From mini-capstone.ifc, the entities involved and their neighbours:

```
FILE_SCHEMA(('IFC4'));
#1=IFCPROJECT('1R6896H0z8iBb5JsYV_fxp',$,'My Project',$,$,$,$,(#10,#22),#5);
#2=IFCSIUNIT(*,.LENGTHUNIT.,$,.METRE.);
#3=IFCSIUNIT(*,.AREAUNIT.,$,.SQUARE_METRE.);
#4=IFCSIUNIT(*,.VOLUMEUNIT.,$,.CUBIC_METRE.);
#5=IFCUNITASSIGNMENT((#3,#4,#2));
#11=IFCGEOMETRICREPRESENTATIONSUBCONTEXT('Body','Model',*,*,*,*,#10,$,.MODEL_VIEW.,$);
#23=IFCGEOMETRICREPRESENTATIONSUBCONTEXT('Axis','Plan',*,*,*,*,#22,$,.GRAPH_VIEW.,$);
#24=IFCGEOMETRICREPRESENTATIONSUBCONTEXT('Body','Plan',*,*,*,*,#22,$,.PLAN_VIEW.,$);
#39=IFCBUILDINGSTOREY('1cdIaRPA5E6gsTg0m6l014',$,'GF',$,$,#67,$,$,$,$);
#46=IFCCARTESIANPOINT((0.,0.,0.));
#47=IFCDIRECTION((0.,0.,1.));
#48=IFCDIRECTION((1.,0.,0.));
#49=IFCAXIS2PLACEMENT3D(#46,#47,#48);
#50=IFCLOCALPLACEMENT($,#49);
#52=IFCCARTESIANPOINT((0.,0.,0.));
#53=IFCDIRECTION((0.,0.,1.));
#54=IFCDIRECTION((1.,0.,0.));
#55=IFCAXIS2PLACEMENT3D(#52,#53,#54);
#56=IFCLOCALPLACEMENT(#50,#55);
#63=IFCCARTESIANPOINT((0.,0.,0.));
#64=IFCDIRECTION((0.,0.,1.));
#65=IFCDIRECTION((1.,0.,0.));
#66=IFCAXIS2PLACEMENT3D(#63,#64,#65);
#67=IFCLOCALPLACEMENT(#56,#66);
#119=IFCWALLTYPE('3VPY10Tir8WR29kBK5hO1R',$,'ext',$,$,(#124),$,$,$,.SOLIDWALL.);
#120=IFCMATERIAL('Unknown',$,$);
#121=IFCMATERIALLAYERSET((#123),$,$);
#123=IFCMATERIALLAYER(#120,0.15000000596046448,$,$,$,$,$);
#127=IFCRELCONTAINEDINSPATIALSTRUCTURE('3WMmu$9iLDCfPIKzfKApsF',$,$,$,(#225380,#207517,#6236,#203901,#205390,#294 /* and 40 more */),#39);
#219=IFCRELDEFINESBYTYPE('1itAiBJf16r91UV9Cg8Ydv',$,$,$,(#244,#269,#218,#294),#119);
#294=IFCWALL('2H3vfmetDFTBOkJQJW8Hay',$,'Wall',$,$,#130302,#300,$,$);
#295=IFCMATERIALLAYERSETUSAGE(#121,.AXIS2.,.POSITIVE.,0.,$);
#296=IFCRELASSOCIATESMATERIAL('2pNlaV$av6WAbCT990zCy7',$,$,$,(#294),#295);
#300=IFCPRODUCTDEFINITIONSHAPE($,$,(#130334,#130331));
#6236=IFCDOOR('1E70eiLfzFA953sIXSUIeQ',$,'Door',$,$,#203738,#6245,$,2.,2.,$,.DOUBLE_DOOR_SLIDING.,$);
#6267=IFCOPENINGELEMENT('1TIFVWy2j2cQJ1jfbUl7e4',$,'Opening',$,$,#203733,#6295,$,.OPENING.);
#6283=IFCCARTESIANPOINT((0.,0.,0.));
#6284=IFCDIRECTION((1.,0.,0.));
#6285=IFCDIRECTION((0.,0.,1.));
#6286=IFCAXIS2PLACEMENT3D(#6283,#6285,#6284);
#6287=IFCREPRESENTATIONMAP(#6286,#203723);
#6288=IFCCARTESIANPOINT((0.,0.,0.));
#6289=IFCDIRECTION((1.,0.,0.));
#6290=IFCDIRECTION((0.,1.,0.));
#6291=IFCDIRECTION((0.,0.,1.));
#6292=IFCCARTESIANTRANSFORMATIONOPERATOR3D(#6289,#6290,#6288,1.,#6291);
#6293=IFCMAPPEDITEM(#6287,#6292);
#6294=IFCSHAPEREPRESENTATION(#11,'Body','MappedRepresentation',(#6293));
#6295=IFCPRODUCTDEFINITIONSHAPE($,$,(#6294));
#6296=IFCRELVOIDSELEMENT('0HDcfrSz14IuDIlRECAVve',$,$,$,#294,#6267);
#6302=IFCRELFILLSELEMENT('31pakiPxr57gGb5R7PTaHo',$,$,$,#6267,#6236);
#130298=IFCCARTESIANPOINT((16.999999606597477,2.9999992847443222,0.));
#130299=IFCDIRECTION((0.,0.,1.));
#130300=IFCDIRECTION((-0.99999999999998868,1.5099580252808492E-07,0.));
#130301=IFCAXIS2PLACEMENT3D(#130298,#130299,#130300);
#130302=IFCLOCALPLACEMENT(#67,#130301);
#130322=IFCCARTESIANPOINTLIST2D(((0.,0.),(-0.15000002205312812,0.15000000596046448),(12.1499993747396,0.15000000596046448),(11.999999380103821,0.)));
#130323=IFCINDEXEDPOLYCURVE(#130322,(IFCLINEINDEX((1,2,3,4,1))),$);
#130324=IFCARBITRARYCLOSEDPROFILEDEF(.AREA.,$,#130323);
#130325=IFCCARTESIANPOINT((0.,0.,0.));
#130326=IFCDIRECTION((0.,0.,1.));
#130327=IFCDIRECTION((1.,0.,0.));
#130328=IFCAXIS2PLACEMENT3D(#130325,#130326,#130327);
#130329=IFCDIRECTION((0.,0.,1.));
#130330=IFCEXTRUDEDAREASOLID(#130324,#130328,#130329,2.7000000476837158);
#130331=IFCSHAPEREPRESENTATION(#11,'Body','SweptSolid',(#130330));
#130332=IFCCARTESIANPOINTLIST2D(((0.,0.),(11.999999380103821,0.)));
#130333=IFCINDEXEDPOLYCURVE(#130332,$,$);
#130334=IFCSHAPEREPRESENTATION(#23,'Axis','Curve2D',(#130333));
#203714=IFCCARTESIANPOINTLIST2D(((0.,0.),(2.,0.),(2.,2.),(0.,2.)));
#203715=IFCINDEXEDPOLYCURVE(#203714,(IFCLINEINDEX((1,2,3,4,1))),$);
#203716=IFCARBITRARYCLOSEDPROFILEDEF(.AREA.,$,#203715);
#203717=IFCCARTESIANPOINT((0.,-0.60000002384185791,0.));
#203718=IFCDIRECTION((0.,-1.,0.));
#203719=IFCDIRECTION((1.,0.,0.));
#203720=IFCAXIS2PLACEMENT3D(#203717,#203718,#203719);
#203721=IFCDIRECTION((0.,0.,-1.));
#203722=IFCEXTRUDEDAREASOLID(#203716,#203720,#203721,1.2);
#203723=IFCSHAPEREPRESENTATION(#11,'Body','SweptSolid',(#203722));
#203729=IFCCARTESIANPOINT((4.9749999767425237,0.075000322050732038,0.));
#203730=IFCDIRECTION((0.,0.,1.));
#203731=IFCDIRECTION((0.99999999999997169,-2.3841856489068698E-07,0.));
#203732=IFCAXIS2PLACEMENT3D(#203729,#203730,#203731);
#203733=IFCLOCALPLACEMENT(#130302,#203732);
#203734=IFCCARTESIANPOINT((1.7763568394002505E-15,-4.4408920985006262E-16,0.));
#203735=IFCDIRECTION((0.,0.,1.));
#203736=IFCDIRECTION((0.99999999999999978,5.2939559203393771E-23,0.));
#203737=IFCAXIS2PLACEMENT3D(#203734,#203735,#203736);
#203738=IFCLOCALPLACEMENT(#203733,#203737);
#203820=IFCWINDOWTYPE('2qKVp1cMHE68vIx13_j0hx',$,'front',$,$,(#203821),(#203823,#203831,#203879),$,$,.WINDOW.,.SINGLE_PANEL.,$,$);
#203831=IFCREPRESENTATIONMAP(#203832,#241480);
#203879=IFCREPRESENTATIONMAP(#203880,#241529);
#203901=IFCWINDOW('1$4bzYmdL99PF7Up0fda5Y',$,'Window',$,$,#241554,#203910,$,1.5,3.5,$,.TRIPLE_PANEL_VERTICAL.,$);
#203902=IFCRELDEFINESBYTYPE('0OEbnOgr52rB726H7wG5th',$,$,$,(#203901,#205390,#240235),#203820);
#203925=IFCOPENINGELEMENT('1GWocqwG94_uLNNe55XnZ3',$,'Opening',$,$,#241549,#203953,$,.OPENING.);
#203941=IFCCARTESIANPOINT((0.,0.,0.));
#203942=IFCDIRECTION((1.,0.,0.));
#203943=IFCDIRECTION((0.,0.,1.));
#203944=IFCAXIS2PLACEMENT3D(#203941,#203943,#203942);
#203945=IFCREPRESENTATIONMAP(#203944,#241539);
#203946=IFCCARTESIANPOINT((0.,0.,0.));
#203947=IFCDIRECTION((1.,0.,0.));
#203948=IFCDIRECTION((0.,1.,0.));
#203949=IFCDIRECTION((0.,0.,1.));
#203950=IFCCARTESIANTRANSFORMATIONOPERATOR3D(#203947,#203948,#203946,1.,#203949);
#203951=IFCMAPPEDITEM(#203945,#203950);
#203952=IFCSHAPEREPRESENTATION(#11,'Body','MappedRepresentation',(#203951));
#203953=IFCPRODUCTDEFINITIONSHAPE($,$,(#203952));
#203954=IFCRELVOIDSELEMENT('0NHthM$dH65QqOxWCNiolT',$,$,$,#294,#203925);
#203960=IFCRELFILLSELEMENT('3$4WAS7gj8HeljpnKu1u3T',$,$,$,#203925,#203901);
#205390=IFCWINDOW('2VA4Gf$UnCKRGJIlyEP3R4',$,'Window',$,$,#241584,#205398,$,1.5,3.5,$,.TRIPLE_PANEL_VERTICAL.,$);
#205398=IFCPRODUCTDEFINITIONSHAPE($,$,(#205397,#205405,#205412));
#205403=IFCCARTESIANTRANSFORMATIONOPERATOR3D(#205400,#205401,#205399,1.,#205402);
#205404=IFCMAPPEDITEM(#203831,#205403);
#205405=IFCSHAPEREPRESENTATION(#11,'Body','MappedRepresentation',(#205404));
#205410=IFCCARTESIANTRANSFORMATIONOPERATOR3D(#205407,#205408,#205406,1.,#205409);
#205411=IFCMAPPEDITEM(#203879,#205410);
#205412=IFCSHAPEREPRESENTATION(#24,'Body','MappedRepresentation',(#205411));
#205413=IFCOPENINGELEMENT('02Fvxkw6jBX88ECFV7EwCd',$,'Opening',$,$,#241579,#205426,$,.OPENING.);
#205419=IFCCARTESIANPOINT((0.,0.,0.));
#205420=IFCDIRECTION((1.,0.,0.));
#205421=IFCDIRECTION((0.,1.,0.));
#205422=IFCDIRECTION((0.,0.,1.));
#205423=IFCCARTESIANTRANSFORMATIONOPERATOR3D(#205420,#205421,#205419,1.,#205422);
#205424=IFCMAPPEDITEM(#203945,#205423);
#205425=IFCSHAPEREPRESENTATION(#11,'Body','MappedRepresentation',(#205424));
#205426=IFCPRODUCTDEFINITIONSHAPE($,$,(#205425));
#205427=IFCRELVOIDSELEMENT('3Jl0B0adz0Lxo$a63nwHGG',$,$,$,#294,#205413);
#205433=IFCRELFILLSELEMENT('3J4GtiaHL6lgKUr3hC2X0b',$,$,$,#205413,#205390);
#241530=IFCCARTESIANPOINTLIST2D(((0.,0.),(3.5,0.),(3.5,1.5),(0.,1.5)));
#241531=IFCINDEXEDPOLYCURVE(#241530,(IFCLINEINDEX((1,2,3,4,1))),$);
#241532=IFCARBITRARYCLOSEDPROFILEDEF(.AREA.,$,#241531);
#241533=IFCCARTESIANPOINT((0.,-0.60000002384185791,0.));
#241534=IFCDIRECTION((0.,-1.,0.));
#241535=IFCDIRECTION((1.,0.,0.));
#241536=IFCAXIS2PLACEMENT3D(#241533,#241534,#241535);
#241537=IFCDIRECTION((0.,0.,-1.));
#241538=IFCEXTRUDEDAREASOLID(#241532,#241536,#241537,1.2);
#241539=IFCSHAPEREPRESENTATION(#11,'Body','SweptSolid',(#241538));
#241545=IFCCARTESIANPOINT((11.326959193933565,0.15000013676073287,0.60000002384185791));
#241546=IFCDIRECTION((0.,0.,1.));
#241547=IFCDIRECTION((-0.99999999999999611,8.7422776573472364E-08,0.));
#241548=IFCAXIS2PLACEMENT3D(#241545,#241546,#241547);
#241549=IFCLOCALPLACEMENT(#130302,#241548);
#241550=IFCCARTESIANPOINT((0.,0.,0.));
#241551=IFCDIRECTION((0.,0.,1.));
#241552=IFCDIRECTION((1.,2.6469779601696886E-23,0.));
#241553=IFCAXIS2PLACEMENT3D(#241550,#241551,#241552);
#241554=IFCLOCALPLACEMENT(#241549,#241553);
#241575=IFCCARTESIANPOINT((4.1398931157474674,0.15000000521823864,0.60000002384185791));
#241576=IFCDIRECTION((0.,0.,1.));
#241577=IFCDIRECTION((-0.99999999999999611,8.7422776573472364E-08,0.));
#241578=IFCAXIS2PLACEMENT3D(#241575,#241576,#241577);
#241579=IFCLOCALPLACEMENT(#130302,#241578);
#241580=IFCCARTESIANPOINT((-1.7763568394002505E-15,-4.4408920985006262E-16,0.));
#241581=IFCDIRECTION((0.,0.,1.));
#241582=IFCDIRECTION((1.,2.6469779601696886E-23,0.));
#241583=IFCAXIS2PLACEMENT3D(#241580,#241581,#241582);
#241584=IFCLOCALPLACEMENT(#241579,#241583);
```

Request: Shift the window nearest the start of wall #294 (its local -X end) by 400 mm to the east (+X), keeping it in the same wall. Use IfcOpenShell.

```python
import ifcopenshell
import ifcopenshell.api.geometry
import ifcopenshell.util.placement

model = ifcopenshell.open("mini-capstone.ifc")

window = model.by_guid("2VA4Gf$UnCKRGJIlyEP3R4")
opening = window.FillsVoids[0].RelatingOpeningElement
wall = opening.VoidsElements[0].RelatingBuildingElement

wall_matrix = ifcopenshell.util.placement.get_local_placement(wall.ObjectPlacement)
shift = wall_matrix[:3, 0] * -0.4
before = ifcopenshell.util.placement.get_local_placement(window.ObjectPlacement)[:3, 3].copy()

# The window is placed relative to its opening, so it follows when the opening moves.
matrix = ifcopenshell.util.placement.get_local_placement(opening.ObjectPlacement)
matrix[:3, 3] += shift
ifcopenshell.api.geometry.edit_object_placement(
    model, product=opening, matrix=matrix, is_si=False, should_transform_children=True
)

after = ifcopenshell.util.placement.get_local_placement(window.ObjectPlacement)[:3, 3]
print("window moved by", (after - before).round(3) + 0.0)

model.write("mini-capstone_edited.ifc")
```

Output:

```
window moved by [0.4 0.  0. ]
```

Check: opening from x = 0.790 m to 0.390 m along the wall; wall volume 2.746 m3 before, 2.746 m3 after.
